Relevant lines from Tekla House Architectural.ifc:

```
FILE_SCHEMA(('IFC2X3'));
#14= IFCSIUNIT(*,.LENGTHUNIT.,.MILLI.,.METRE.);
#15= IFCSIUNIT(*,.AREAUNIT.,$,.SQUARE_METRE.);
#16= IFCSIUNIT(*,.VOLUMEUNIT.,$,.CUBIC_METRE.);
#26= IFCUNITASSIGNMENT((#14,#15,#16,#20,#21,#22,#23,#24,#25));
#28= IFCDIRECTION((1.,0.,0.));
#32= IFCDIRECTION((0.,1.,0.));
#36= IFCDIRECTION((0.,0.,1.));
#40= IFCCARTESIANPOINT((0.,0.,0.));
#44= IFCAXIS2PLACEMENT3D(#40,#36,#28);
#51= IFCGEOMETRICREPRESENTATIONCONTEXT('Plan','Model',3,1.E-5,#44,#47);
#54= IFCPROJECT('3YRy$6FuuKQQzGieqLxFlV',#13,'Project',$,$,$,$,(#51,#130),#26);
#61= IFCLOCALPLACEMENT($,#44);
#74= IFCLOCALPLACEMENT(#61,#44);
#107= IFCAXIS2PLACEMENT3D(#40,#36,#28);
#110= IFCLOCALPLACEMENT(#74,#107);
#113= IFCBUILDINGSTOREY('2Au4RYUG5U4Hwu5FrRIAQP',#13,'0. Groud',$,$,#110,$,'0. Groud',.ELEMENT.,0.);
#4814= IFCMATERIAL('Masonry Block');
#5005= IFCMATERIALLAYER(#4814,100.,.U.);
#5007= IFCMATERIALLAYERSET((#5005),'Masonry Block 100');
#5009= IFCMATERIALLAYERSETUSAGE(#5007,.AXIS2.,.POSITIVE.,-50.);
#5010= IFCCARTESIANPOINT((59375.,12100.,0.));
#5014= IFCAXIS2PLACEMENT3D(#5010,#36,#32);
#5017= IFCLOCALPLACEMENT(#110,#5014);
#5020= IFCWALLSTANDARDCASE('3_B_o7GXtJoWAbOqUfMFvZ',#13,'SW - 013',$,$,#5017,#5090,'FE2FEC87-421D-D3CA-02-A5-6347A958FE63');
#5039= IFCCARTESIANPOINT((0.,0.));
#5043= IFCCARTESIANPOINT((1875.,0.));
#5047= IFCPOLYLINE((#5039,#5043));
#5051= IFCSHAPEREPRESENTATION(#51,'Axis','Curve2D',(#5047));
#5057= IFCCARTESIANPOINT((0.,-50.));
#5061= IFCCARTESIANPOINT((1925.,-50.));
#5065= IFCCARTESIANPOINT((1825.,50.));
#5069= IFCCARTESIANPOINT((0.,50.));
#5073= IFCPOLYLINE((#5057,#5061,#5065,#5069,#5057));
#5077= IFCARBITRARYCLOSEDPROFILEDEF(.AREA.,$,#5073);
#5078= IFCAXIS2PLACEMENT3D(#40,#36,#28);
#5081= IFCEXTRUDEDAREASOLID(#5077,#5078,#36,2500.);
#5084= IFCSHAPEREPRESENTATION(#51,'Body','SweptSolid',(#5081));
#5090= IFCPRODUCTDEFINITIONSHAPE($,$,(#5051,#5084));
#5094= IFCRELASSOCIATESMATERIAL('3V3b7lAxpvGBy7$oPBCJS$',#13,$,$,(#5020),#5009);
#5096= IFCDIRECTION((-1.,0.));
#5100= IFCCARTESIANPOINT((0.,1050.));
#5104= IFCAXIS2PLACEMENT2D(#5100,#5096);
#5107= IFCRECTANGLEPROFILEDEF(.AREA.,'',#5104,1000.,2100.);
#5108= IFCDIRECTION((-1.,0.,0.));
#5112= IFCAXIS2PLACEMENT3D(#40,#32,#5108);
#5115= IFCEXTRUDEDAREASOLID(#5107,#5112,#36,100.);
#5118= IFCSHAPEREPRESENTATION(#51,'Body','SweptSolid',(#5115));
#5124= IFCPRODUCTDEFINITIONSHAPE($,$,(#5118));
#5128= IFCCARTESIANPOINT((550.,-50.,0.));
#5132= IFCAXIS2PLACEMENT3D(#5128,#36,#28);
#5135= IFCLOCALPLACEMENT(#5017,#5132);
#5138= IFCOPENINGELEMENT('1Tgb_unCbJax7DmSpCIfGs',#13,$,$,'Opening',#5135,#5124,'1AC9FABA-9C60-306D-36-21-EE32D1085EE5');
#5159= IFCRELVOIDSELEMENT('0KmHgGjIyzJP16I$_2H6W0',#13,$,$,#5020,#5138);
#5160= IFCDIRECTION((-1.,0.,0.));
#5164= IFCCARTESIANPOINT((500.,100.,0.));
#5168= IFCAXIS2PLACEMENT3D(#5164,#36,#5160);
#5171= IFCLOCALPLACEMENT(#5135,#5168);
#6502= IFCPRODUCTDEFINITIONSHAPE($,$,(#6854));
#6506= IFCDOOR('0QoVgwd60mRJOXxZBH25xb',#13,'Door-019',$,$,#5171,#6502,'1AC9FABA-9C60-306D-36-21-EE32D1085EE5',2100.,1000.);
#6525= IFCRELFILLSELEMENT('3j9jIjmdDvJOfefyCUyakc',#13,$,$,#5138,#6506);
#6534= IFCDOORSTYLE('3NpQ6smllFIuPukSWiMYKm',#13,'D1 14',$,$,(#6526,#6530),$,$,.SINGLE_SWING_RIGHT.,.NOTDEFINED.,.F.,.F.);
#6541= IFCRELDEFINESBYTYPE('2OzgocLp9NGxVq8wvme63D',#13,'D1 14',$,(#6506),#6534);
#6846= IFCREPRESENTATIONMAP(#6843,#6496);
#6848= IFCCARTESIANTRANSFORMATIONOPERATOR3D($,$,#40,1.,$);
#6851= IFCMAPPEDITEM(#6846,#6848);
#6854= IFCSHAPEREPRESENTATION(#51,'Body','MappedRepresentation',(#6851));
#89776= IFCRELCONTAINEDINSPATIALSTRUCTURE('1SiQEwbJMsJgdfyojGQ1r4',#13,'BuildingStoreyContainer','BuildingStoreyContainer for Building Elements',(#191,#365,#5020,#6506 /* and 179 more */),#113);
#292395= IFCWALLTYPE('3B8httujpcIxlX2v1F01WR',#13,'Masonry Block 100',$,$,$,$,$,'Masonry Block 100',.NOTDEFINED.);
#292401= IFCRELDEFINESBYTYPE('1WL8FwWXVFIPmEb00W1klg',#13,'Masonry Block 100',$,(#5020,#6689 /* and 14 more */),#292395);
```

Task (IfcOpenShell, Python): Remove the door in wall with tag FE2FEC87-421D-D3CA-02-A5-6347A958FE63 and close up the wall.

```python
import ifcopenshell
import ifcopenshell.api.feature
import ifcopenshell.api.root
import ifcopenshell.geom
import ifcopenshell.util.shape

model = ifcopenshell.open("Tekla House Architectural.ifc")
settings = ifcopenshell.geom.settings()


def volume(element):
    """Net volume in cubic metres, openings subtracted."""
    shape = ifcopenshell.geom.create_shape(settings, element)
    return ifcopenshell.util.shape.get_volume(shape.geometry)


door = model.by_guid("0QoVgwd60mRJOXxZBH25xb")
opening = door.FillsVoids[0].RelatingOpeningElement
wall = opening.VoidsElements[0].RelatingBuildingElement
before = volume(wall)

ifcopenshell.api.root.remove_product(model, product=door)
ifcopenshell.api.feature.remove_feature(model, feature=opening)

after = volume(wall)

print(f"wall volume {before:.3f} -> {after:.3f} m3")

model.write("Tekla House Architectural_edited.ifc")
```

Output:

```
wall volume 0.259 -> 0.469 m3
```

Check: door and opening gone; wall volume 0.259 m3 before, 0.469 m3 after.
